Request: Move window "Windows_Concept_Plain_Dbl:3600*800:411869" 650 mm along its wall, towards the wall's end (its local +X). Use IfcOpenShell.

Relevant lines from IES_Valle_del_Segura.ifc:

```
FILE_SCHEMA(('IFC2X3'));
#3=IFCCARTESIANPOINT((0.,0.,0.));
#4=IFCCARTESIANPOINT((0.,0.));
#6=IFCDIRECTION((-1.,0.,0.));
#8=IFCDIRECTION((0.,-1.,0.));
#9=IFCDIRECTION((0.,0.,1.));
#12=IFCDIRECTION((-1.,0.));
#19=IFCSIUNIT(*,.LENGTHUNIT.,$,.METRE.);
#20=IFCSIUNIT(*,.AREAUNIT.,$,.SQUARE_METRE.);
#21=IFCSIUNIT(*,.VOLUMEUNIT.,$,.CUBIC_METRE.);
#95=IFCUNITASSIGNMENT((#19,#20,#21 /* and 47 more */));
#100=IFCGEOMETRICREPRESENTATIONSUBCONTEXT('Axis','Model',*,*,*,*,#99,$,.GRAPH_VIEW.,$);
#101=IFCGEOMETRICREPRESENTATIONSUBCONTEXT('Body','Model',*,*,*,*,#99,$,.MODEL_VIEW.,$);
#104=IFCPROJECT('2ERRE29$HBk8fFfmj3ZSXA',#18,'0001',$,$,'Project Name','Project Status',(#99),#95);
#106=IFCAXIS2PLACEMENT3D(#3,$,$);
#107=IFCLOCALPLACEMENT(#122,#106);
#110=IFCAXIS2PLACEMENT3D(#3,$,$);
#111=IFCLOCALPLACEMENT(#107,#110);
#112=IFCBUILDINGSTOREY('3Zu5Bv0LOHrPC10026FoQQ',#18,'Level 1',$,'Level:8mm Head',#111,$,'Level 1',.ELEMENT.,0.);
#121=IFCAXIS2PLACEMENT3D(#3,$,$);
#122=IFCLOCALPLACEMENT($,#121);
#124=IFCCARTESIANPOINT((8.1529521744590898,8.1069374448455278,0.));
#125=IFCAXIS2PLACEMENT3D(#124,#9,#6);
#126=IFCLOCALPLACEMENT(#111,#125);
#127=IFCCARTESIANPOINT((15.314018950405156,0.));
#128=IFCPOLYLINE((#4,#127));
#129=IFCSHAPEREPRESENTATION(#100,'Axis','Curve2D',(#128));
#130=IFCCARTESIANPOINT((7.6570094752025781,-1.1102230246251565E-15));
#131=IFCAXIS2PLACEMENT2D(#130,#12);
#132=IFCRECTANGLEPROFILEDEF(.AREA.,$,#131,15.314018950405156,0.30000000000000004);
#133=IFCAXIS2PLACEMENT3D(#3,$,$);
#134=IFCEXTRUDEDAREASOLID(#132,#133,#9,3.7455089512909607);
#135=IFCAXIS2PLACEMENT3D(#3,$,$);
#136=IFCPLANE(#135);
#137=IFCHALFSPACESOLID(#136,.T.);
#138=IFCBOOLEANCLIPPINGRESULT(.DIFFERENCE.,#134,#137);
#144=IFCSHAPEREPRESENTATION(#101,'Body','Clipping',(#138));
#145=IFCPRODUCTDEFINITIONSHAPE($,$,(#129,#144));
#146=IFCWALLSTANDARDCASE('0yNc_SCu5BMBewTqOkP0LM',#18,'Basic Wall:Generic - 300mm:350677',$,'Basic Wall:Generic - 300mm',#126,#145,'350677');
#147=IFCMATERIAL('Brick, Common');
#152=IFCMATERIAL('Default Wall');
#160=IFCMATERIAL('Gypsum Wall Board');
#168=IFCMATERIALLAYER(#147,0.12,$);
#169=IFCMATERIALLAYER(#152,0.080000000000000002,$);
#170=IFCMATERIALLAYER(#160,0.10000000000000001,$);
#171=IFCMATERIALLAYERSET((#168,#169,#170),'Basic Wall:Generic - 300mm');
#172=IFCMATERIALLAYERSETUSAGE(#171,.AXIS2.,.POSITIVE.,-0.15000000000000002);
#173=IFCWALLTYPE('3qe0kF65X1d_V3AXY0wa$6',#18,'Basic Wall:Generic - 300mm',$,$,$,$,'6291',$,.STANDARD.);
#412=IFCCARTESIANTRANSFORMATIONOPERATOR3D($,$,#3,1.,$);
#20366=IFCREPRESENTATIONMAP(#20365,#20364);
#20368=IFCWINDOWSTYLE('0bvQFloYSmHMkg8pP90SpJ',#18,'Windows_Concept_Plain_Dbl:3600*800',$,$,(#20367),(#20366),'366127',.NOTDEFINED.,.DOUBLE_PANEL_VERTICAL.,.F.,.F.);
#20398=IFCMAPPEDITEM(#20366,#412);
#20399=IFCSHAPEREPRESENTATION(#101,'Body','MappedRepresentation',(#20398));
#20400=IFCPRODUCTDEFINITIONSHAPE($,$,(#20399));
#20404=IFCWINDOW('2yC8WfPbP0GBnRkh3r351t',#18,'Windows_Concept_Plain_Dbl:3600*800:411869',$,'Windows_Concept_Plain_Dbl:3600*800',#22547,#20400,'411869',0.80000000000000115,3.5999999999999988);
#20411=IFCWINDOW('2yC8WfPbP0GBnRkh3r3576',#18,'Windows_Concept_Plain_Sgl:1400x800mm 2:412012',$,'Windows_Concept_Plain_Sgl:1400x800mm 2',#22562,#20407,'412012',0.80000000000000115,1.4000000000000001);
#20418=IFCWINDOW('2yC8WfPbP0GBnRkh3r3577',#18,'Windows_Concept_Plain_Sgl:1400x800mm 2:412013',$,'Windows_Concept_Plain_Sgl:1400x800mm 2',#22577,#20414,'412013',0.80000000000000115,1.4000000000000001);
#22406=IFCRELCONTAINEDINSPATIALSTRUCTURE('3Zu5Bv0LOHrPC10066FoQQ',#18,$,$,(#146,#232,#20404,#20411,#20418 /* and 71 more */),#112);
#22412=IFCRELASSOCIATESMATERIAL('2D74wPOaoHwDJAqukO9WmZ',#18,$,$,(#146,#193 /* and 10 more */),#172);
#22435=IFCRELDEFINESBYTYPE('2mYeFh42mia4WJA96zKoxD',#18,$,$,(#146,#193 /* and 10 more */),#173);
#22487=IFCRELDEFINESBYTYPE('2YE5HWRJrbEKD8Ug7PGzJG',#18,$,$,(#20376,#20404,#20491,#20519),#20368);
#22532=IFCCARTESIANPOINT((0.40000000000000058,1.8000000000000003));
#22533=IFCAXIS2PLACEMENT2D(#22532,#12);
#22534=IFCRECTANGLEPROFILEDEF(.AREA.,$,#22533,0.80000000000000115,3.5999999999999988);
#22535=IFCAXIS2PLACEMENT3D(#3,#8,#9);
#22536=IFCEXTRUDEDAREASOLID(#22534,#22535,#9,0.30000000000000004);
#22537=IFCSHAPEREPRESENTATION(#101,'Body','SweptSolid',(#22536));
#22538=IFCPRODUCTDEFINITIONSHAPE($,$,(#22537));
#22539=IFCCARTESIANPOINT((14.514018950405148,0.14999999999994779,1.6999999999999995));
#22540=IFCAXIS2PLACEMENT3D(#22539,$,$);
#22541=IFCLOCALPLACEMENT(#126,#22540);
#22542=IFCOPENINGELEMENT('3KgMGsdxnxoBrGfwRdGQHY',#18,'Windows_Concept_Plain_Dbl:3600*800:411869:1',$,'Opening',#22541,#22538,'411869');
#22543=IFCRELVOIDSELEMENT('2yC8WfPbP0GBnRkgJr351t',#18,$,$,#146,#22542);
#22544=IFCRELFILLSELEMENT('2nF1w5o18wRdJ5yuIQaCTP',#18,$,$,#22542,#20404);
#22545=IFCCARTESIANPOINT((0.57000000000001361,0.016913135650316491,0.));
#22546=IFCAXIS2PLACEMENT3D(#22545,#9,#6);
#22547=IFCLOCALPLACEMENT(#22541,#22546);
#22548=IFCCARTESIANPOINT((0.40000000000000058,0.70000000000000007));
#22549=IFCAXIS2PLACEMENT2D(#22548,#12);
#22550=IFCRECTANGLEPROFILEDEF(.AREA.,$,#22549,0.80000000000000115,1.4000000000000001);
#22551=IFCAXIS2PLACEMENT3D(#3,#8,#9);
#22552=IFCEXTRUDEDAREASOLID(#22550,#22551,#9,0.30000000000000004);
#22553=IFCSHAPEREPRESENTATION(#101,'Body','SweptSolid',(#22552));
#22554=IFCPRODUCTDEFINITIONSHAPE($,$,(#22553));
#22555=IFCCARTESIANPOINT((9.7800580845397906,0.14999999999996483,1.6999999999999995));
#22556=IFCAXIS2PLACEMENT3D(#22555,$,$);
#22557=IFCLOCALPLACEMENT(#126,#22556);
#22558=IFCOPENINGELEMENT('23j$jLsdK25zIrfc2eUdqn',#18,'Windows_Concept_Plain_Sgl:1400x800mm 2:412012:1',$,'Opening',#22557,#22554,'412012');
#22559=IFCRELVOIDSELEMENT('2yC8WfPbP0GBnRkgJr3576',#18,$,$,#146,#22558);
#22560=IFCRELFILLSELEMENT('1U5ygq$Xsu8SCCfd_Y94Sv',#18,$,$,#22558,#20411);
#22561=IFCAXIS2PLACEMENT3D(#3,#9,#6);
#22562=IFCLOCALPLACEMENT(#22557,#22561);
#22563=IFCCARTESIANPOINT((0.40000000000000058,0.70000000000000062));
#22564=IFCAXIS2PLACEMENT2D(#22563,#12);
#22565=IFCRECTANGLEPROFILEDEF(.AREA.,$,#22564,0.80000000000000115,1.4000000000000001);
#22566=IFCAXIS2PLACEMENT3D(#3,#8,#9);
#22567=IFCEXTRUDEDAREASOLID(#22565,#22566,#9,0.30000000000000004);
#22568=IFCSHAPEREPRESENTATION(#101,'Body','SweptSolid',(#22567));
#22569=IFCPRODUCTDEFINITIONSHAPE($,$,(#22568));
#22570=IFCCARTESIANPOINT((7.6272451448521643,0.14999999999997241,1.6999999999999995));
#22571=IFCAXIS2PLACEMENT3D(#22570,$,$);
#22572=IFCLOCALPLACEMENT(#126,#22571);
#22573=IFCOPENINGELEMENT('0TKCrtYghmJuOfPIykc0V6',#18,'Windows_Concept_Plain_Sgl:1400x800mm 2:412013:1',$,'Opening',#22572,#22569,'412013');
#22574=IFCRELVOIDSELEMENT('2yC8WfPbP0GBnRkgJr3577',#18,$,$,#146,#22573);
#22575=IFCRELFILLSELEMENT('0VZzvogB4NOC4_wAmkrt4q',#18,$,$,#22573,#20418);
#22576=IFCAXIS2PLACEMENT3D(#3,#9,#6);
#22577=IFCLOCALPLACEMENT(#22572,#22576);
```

```python
import ifcopenshell
import ifcopenshell.api.geometry
import ifcopenshell.util.placement
import ifcopenshell.util.unit

model = ifcopenshell.open("IES_Valle_del_Segura.ifc")
unit_scale = ifcopenshell.util.unit.calculate_unit_scale(model)

window = model.by_id(20404)
opening = window.FillsVoids[0].RelatingOpeningElement
wall = opening.VoidsElements[0].RelatingBuildingElement

wall_matrix = ifcopenshell.util.placement.get_local_placement(wall.ObjectPlacement)
shift = wall_matrix[:3, 0] * 0.65 / unit_scale
before = ifcopenshell.util.placement.get_local_placement(window.ObjectPlacement)[:3, 3].copy()

# The window is placed relative to its opening, so it follows when the opening moves.
matrix = ifcopenshell.util.placement.get_local_placement(opening.ObjectPlacement)
matrix[:3, 3] += shift
ifcopenshell.api.geometry.edit_object_placement(
    model, product=opening, matrix=matrix, is_si=False, should_transform_children=True
)

after = ifcopenshell.util.placement.get_local_placement(window.ObjectPlacement)[:3, 3]
print("window moved by", (after - before).round(3) + 0.0)

model.write("IES_Valle_del_Segura-out.ifc")
```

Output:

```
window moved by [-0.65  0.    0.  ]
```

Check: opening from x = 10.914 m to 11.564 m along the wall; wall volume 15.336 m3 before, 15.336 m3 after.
